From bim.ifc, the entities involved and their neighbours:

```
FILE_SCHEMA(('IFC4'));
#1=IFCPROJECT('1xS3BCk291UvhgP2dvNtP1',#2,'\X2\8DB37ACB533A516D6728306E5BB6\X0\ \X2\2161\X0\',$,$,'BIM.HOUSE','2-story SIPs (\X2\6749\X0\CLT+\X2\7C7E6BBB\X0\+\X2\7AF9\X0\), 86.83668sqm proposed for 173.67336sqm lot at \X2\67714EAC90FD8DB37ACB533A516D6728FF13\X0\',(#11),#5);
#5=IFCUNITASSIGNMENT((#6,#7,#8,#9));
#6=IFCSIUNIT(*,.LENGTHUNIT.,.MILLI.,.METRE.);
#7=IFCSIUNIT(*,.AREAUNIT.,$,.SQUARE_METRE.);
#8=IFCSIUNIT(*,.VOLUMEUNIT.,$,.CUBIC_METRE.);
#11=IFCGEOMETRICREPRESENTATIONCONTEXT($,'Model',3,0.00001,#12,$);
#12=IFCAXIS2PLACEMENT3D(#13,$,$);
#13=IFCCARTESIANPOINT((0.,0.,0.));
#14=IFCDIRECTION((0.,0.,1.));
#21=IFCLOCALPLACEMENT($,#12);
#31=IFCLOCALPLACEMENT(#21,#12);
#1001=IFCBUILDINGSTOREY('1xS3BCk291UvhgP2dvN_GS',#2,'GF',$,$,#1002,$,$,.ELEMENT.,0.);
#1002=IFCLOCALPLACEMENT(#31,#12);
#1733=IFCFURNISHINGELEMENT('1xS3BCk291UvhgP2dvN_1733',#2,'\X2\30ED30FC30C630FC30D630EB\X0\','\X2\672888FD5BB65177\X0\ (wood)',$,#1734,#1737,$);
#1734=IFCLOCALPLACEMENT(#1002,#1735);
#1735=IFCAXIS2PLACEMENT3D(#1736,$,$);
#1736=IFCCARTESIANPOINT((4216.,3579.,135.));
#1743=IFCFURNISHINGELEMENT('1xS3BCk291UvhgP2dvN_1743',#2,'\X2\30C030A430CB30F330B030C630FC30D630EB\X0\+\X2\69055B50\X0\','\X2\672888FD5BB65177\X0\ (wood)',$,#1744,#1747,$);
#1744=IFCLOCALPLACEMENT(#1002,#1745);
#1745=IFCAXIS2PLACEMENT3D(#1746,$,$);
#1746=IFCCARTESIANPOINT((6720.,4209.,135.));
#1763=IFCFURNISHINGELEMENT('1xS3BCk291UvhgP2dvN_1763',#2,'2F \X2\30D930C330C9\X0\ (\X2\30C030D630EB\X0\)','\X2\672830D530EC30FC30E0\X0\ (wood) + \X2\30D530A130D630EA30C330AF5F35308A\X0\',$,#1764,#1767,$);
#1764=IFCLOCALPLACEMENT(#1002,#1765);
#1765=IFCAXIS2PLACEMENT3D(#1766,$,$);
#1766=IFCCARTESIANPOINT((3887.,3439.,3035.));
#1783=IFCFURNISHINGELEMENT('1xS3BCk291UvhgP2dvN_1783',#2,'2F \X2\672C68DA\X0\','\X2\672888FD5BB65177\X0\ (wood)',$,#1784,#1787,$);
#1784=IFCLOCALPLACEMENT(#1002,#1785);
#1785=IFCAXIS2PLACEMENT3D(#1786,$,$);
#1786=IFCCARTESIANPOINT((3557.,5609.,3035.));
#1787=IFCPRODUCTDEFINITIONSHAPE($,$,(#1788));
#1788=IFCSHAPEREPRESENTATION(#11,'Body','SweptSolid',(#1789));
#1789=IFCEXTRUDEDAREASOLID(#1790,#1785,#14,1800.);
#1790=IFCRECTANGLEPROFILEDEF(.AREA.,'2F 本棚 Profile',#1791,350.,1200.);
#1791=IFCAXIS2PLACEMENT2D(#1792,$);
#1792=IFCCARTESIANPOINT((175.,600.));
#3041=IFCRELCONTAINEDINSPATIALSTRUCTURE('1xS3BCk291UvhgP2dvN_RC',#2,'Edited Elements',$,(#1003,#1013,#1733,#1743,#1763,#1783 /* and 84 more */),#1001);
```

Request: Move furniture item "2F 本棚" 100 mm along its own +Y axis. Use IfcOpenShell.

```python
import ifcopenshell
import ifcopenshell.api.geometry
import ifcopenshell.util.placement

model = ifcopenshell.open("bim.ifc")

item = model.by_guid("1xS3BCk291UvhgP2dvN_1783")
matrix = ifcopenshell.util.placement.get_local_placement(item.ObjectPlacement)
matrix[:3, 3] += matrix[:3, 1] * 100.0
ifcopenshell.api.geometry.edit_object_placement(model, product=item, matrix=matrix, is_si=False)

print(ifcopenshell.util.placement.get_local_placement(item.ObjectPlacement).round(3) + 0.0)

model.write("bim_updated.ifc")
```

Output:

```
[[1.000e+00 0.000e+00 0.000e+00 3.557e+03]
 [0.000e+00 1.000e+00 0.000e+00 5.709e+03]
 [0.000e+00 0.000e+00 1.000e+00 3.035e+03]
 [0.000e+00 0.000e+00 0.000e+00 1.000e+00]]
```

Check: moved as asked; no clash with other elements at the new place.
